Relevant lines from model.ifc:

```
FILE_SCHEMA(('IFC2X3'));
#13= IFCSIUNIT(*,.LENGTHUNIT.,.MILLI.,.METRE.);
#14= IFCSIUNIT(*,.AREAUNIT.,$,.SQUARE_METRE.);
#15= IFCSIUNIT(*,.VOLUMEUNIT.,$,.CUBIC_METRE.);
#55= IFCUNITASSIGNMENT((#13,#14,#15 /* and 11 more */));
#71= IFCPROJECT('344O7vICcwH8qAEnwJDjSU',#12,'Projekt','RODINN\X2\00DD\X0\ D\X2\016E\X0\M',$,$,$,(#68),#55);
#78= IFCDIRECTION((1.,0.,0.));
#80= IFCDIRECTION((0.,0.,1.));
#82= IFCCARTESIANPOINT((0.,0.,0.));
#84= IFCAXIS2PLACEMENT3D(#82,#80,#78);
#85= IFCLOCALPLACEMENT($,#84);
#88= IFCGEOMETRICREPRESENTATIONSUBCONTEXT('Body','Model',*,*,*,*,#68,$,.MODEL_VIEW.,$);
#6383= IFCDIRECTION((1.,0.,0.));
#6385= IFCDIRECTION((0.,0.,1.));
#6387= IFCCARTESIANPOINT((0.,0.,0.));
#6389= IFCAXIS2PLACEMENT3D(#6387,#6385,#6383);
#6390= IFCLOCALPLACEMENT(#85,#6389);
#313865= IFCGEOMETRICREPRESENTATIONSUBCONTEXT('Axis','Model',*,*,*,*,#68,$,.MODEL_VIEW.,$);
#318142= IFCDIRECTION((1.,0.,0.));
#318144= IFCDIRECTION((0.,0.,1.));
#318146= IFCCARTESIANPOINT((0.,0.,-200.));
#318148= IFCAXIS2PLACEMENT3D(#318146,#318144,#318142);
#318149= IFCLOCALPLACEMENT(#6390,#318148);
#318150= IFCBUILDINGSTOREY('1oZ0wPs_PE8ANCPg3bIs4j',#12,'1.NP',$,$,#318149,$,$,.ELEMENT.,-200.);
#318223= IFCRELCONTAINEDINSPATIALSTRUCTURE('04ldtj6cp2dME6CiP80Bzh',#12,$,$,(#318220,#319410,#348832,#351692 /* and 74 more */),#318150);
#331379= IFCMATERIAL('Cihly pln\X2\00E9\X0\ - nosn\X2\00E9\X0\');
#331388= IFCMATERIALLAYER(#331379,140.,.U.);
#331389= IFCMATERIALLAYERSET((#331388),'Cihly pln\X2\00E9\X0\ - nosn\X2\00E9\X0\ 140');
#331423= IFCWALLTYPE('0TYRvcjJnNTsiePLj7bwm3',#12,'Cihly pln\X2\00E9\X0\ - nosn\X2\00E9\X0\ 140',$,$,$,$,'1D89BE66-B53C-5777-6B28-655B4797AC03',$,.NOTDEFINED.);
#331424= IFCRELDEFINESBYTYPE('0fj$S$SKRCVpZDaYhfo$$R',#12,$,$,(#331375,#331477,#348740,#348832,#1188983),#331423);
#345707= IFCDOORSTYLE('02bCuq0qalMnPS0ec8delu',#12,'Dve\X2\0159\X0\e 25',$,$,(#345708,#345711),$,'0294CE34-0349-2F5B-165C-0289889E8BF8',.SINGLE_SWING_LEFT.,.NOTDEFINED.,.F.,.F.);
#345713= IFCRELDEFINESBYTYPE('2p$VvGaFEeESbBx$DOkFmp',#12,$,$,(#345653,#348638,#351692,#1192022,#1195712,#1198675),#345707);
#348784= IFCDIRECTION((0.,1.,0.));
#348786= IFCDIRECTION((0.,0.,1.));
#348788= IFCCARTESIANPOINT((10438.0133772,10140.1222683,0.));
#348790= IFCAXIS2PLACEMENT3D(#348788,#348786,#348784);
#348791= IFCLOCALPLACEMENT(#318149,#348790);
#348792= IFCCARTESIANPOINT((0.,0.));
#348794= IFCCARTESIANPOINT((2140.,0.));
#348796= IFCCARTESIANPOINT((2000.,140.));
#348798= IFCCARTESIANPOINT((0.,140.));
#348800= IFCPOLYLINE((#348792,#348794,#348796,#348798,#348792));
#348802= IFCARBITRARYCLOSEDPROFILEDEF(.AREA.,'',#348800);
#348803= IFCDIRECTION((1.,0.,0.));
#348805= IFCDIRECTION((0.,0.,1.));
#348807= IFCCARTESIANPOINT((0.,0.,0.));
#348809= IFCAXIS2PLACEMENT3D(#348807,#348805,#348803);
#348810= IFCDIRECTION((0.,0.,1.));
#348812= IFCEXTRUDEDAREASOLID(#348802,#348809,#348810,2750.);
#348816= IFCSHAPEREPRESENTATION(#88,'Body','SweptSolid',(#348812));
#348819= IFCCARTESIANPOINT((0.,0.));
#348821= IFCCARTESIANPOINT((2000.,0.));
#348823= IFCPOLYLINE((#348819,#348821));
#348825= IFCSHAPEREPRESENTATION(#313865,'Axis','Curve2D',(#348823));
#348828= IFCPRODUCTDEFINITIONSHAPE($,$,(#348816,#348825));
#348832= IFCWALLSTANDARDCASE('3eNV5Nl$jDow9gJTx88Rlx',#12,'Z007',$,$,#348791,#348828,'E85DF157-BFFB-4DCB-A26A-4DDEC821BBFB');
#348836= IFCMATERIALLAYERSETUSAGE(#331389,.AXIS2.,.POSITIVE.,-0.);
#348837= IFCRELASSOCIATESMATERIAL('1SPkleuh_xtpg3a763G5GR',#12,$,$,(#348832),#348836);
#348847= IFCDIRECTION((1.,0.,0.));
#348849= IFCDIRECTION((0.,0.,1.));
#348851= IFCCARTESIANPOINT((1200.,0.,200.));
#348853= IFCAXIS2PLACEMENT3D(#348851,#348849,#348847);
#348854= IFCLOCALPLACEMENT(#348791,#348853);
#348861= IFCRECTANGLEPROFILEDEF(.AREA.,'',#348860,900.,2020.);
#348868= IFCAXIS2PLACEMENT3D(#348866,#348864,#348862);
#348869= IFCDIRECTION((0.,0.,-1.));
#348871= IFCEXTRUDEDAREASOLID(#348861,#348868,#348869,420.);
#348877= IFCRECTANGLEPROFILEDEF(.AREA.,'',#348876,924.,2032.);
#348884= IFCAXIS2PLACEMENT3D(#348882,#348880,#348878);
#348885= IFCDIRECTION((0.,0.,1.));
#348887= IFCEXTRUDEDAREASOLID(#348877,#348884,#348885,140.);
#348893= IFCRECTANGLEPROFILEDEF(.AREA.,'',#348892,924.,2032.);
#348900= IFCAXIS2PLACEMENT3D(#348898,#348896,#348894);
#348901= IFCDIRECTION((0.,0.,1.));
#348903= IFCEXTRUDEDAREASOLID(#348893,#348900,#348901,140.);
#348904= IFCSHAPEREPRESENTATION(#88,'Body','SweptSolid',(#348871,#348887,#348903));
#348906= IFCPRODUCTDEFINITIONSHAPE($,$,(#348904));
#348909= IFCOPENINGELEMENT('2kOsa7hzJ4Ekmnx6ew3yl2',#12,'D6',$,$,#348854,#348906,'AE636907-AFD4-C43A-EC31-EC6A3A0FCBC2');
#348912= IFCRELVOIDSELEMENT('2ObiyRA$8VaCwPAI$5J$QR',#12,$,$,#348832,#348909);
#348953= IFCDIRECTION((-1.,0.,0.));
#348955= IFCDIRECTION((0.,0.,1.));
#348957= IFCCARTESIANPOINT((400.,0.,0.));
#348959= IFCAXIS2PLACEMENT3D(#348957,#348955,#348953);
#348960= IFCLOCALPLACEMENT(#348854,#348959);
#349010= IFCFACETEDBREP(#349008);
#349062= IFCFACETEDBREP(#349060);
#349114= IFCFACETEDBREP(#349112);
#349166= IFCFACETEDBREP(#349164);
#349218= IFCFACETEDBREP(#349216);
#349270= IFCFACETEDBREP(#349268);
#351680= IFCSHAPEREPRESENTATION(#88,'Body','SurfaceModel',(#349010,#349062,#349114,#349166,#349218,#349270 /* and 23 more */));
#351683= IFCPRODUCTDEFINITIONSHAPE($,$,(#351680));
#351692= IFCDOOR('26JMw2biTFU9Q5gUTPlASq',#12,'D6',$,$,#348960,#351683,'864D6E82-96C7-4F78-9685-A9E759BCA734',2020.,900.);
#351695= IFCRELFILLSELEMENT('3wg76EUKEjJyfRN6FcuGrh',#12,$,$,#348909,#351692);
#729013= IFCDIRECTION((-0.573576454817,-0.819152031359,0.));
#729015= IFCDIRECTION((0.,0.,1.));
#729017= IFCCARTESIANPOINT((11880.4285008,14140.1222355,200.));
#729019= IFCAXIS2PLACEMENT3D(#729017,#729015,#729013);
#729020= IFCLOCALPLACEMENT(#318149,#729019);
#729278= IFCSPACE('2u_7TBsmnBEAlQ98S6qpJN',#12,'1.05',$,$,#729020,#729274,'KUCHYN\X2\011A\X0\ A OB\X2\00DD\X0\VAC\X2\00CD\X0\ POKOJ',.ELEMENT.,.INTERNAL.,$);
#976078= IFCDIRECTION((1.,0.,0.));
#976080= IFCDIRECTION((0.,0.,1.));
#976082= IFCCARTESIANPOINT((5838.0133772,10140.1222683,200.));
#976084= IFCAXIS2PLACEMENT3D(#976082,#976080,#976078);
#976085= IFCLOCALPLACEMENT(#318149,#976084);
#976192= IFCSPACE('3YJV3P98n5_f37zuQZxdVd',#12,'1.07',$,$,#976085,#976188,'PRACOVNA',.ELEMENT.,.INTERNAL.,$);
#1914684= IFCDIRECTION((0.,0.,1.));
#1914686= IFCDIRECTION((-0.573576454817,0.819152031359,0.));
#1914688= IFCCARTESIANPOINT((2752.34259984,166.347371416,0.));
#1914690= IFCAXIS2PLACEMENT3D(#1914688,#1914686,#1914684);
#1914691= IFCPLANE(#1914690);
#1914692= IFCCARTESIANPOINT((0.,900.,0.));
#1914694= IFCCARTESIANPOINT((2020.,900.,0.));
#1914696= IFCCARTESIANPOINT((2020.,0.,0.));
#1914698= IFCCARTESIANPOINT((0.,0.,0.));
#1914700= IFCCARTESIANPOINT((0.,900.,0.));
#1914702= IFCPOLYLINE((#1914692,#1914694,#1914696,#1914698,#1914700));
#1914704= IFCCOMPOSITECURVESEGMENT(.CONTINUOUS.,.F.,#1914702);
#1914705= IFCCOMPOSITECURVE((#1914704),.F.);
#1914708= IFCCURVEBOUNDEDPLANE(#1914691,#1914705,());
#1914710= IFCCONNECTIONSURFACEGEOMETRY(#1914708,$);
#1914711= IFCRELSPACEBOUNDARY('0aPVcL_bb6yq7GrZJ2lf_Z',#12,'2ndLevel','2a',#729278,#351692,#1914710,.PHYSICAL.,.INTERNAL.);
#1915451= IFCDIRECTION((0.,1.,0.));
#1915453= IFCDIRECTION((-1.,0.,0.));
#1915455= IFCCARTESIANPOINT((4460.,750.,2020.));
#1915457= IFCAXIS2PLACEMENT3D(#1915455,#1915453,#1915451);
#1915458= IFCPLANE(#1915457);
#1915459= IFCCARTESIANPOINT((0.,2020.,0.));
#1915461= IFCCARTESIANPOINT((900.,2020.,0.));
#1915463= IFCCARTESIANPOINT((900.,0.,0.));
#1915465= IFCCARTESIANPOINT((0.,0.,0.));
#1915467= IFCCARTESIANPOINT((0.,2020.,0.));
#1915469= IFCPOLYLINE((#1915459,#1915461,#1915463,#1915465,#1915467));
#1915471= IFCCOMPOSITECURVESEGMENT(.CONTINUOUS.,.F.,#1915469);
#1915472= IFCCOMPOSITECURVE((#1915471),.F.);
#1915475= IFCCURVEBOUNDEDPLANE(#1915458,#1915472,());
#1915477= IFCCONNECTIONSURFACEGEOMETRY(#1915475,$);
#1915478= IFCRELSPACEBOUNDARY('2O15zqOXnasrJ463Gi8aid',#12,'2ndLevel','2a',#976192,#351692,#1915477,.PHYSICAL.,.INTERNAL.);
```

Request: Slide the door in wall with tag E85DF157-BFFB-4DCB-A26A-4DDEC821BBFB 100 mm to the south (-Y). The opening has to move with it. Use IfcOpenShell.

```python
import numpy as np
import ifcopenshell
import ifcopenshell.api.geometry
import ifcopenshell.util.placement
import ifcopenshell.util.unit

model = ifcopenshell.open("model.ifc")
unit_scale = ifcopenshell.util.unit.calculate_unit_scale(model)

door = model.by_guid("26JMw2biTFU9Q5gUTPlASq")
opening = door.FillsVoids[0].RelatingOpeningElement
wall = opening.VoidsElements[0].RelatingBuildingElement

wall_matrix = ifcopenshell.util.placement.get_local_placement(wall.ObjectPlacement)
shift = wall_matrix[:3, 0] * -0.1 / unit_scale
before = ifcopenshell.util.placement.get_local_placement(door.ObjectPlacement)[:3, 3].copy()

# The door is placed relative to its opening, so it follows when the opening moves.
matrix = ifcopenshell.util.placement.get_local_placement(opening.ObjectPlacement)
matrix[:3, 3] += shift
ifcopenshell.api.geometry.edit_object_placement(
    model, product=opening, matrix=matrix, is_si=False, should_transform_children=True
)

# Space boundary surfaces are stored in each space's coordinates; move them too.
for rel in door.ProvidesBoundaries:
    if not rel.ConnectionGeometry:
        continue
    surface = rel.ConnectionGeometry.SurfaceOnRelatingElement.BasisSurface
    space_matrix = ifcopenshell.util.placement.get_local_placement(rel.RelatingSpace.ObjectPlacement)
    point = np.array(surface.Position.Location.Coordinates) + space_matrix[:3, :3].T @ shift
    surface.Position = model.createIfcAxis2Placement3D(
        model.createIfcCartesianPoint(point.tolist()), surface.Position.Axis, surface.Position.RefDirection
    )

after = ifcopenshell.util.placement.get_local_placement(door.ObjectPlacement)[:3, 3]
print("door moved by", (after - before).round(3) + 0.0)

model.write("model_updated.ifc")
```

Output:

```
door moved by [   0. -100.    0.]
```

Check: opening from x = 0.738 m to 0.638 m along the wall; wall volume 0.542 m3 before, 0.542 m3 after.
